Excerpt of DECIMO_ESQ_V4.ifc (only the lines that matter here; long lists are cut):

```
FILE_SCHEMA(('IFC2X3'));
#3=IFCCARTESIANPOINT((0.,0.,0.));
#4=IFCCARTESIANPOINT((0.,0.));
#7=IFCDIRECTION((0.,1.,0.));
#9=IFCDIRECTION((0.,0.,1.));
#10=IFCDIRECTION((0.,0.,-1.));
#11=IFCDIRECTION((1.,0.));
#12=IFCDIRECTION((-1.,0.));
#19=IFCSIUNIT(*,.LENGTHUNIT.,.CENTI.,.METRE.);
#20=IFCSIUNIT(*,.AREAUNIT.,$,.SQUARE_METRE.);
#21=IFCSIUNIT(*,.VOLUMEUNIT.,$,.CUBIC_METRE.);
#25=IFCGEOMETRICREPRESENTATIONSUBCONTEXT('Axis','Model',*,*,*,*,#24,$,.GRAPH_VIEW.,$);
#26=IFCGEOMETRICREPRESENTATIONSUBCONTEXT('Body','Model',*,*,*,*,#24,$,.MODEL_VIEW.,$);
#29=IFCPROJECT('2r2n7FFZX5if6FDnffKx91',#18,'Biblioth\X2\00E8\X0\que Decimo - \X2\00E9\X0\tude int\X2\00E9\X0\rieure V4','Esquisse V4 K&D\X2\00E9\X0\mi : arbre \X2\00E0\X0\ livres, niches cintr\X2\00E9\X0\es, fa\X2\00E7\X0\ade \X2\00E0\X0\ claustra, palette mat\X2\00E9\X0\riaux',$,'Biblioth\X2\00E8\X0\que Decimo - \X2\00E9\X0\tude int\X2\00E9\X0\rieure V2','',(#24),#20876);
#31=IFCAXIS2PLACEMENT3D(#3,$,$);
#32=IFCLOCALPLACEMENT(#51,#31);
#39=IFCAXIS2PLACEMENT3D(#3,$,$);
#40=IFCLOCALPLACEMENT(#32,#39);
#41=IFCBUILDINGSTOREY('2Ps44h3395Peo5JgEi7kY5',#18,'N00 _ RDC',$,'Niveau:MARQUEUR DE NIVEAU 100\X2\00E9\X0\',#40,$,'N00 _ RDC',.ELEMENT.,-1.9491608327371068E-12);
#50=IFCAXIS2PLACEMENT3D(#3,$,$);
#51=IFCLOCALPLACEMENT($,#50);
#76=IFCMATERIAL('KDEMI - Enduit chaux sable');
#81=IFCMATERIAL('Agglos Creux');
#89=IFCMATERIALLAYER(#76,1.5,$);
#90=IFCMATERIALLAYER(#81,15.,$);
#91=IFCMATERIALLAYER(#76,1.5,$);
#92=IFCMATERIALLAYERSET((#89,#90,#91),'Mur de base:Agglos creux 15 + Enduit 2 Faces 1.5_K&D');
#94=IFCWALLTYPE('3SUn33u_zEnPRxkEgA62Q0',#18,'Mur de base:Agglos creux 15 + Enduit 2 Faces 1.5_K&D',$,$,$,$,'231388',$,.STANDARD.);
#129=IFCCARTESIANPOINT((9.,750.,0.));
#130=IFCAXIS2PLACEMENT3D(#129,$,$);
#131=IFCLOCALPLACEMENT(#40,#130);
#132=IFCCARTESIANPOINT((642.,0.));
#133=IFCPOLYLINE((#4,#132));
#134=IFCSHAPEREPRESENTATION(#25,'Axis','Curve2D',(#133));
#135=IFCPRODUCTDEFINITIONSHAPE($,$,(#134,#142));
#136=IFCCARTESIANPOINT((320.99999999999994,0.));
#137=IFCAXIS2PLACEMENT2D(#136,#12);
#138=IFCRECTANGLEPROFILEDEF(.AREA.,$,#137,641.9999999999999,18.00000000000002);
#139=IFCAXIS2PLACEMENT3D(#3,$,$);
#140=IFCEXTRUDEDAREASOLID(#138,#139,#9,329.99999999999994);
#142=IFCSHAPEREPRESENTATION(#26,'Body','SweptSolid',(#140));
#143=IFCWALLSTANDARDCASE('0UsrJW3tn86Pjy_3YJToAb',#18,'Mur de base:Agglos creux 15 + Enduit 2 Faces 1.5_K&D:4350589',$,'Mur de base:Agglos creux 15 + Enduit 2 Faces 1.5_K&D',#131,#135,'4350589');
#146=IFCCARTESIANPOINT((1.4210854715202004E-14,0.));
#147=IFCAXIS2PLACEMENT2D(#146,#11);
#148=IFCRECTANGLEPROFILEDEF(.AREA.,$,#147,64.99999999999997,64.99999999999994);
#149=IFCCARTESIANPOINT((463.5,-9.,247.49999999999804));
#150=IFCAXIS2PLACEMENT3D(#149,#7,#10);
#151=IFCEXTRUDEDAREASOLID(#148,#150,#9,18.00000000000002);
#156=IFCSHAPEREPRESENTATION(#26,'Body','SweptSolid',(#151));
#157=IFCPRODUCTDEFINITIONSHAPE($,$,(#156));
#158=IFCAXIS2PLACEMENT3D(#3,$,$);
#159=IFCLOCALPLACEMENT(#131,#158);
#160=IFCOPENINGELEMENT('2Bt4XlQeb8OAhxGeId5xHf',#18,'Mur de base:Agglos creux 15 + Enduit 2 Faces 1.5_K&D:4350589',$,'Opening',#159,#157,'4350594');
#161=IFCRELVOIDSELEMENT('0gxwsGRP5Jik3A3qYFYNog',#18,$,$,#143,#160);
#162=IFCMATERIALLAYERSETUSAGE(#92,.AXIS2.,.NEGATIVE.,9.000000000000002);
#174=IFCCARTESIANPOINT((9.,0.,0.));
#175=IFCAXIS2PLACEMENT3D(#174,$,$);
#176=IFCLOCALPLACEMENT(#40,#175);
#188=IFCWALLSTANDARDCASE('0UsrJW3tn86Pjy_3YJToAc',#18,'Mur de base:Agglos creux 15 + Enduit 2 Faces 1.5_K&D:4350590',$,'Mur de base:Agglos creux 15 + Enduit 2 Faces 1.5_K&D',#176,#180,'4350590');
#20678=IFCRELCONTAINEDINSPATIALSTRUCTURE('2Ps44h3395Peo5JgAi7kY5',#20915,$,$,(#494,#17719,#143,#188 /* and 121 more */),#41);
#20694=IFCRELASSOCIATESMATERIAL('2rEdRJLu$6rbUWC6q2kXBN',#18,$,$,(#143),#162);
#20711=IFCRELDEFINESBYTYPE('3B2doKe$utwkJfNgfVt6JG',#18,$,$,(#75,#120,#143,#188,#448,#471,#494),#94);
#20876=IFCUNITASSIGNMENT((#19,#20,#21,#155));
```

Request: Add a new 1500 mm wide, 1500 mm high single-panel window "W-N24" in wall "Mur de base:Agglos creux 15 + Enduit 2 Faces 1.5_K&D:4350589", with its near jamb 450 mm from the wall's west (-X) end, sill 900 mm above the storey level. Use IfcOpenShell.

```python
import numpy as np
import ifcopenshell
import ifcopenshell.api.feature
import ifcopenshell.api.geometry
import ifcopenshell.api.root
import ifcopenshell.api.spatial
import ifcopenshell.api.type
import ifcopenshell.geom
import ifcopenshell.util.element
import ifcopenshell.util.placement
import ifcopenshell.util.representation
import ifcopenshell.util.shape
import ifcopenshell.util.unit

model = ifcopenshell.open("DECIMO_ESQ_V4.ifc")
unit_scale = ifcopenshell.util.unit.calculate_unit_scale(model)
settings = ifcopenshell.geom.settings()


def volume(element):
    """Net volume in cubic metres, openings subtracted."""
    shape = ifcopenshell.geom.create_shape(settings, element)
    return ifcopenshell.util.shape.get_volume(shape.geometry)


wall = model.by_id(143)
storey = ifcopenshell.util.element.get_container(wall, ifc_class="IfcBuildingStorey")
context = ifcopenshell.util.representation.get_context(model, "Model", "Body", "MODEL_VIEW")
before = volume(wall)

width, height, from_end, sill = 1.5, 1.5, 0.45, 0.9  # metres

# The wall runs along its own X axis, and the end named is its -X end.
wall_shape = ifcopenshell.geom.create_shape(settings, wall)
x, y, z = ifcopenshell.util.shape.get_vertices(wall_shape.geometry).T
start = x.min() + from_end
face, thickness = float(y.min()), float(y.max() - y.min())
wall_matrix = ifcopenshell.util.placement.get_local_placement(wall.ObjectPlacement)
level = ifcopenshell.util.placement.get_local_placement(storey.ObjectPlacement)[2, 3]


def in_wall(x, y):
    """Placement at x, y metres in the wall's axes, at sill height."""
    matrix = wall_matrix.copy()
    matrix[:, 3] = wall_matrix @ np.array([x / unit_scale, y / unit_scale, 0.0, 1.0])
    matrix[2, 3] = level + sill / unit_scale
    return matrix


# Opening: a box that overshoots both wall faces by 50 mm.
opening = ifcopenshell.api.root.create_entity(model, ifc_class="IfcOpeningElement")
box = ifcopenshell.api.geometry.add_wall_representation(
    model, context=context, length=width, height=height, thickness=thickness + 0.1
)
ifcopenshell.api.geometry.assign_representation(model, product=opening, representation=box)
ifcopenshell.api.geometry.edit_object_placement(model, product=opening, matrix=in_wall(start, face - 0.05), is_si=False)
ifcopenshell.api.feature.add_feature(model, feature=opening, element=wall)

window = ifcopenshell.api.root.create_entity(model, ifc_class="IfcWindow", name="W-N24")
window.OverallWidth, window.OverallHeight = width / unit_scale, height / unit_scale
body = ifcopenshell.api.geometry.add_window_representation(
    model,
    context=context,
    overall_width=window.OverallWidth,
    overall_height=window.OverallHeight,
    partition_type="SINGLE_PANEL",
)
ifcopenshell.api.geometry.assign_representation(model, product=window, representation=body)
ifcopenshell.api.spatial.assign_container(model, products=[window], relating_structure=storey)
fills = ifcopenshell.api.feature.add_filling(model, opening=opening, element=window)
fills.OwnerHistory = window.OwnerHistory  # required in IFC2X3

# IFC2X3 keeps the operation on the window style.
style = ifcopenshell.api.root.create_entity(model, ifc_class="IfcWindowStyle", name="W-N24")
style.OperationType, style.ConstructionType = "SINGLE_PANEL", "NOTDEFINED"
style.ParameterTakesPrecedence = style.Sizeable = False
ifcopenshell.api.type.assign_type(model, related_objects=[window], relating_type=style)

# Centre the window in the wall's thickness.
ifcopenshell.api.geometry.edit_object_placement(model, product=window, matrix=in_wall(start, face), is_si=False)
window_shape = ifcopenshell.geom.create_shape(settings, window)
depth = ifcopenshell.util.shape.get_vertices(window_shape.geometry)[:, 1]
offset = face + thickness / 2 - (depth.min() + depth.max()) / 2
ifcopenshell.api.geometry.edit_object_placement(model, product=window, matrix=in_wall(start, offset), is_si=False)

after = volume(wall)

print(f"wall volume {before:.3f} -> {after:.3f} m3")

model.write("DECIMO_ESQ_V4_edited.ifc")
```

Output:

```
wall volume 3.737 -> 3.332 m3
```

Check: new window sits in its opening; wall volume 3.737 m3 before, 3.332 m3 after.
